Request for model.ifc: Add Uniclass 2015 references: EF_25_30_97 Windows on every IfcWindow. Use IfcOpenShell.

First a look at what the model holds.

```python
import ifcopenshell

model = ifcopenshell.open("model.ifc")
print(model.schema)
print("classifications:", [c.Name for c in model.by_type("IfcClassification")])
for ifc_class in ("IfcDoor", "IfcRoof", "IfcStair", "IfcWall", "IfcWindow"):
    print(ifc_class, len(model.by_type(ifc_class)))
```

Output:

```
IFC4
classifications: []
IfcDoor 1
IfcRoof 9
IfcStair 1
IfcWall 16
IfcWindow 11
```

```python
import ifcopenshell
import ifcopenshell.api.classification

model = ifcopenshell.open("model.ifc")

system = ifcopenshell.api.classification.add_classification(model, classification="Uniclass 2015")

codes = {
    "IfcWindow": ("EF_25_30_97", "Windows"),
}
for ifc_class, (code, name) in codes.items():
    products = model.by_type(ifc_class)
    ifcopenshell.api.classification.add_reference(
        model, products=products, classification=system, identification=code, name=name
    )
    print(code, len(products))

model.write("model_rev.ifc")
```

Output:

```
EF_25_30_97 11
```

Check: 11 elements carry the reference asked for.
